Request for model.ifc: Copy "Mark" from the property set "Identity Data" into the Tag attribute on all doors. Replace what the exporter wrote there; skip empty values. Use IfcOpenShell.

First a look at what the model holds.

```python
import ifcopenshell
import ifcopenshell.util.element

model = ifcopenshell.open("model.ifc")
print(model.schema)
doors = model.by_type("IfcDoor")
print(len(doors), "doors")
for e in doors[:8]:
    source = ifcopenshell.util.element.get_pset(e, "Identity Data", "Mark")
    target = e.Tag
    print(e.id(), repr(source), repr(target), sep=" | ")
```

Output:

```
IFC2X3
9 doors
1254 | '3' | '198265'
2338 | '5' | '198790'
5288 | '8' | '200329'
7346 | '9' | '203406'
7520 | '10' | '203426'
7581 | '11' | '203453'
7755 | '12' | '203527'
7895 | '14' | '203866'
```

```python
import ifcopenshell
import ifcopenshell.util.element

model = ifcopenshell.open("model.ifc")

count = 0
for e in model.by_type("IfcDoor"):
    value = ifcopenshell.util.element.get_pset(e, "Identity Data", "Mark")
    current = e.Tag
    if not value or not value.strip() or current == value:
        continue
    e.Tag = value
    count += 1

print(count, "doors updated")

model.write("model-out.ifc")
```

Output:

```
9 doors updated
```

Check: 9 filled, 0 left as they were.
